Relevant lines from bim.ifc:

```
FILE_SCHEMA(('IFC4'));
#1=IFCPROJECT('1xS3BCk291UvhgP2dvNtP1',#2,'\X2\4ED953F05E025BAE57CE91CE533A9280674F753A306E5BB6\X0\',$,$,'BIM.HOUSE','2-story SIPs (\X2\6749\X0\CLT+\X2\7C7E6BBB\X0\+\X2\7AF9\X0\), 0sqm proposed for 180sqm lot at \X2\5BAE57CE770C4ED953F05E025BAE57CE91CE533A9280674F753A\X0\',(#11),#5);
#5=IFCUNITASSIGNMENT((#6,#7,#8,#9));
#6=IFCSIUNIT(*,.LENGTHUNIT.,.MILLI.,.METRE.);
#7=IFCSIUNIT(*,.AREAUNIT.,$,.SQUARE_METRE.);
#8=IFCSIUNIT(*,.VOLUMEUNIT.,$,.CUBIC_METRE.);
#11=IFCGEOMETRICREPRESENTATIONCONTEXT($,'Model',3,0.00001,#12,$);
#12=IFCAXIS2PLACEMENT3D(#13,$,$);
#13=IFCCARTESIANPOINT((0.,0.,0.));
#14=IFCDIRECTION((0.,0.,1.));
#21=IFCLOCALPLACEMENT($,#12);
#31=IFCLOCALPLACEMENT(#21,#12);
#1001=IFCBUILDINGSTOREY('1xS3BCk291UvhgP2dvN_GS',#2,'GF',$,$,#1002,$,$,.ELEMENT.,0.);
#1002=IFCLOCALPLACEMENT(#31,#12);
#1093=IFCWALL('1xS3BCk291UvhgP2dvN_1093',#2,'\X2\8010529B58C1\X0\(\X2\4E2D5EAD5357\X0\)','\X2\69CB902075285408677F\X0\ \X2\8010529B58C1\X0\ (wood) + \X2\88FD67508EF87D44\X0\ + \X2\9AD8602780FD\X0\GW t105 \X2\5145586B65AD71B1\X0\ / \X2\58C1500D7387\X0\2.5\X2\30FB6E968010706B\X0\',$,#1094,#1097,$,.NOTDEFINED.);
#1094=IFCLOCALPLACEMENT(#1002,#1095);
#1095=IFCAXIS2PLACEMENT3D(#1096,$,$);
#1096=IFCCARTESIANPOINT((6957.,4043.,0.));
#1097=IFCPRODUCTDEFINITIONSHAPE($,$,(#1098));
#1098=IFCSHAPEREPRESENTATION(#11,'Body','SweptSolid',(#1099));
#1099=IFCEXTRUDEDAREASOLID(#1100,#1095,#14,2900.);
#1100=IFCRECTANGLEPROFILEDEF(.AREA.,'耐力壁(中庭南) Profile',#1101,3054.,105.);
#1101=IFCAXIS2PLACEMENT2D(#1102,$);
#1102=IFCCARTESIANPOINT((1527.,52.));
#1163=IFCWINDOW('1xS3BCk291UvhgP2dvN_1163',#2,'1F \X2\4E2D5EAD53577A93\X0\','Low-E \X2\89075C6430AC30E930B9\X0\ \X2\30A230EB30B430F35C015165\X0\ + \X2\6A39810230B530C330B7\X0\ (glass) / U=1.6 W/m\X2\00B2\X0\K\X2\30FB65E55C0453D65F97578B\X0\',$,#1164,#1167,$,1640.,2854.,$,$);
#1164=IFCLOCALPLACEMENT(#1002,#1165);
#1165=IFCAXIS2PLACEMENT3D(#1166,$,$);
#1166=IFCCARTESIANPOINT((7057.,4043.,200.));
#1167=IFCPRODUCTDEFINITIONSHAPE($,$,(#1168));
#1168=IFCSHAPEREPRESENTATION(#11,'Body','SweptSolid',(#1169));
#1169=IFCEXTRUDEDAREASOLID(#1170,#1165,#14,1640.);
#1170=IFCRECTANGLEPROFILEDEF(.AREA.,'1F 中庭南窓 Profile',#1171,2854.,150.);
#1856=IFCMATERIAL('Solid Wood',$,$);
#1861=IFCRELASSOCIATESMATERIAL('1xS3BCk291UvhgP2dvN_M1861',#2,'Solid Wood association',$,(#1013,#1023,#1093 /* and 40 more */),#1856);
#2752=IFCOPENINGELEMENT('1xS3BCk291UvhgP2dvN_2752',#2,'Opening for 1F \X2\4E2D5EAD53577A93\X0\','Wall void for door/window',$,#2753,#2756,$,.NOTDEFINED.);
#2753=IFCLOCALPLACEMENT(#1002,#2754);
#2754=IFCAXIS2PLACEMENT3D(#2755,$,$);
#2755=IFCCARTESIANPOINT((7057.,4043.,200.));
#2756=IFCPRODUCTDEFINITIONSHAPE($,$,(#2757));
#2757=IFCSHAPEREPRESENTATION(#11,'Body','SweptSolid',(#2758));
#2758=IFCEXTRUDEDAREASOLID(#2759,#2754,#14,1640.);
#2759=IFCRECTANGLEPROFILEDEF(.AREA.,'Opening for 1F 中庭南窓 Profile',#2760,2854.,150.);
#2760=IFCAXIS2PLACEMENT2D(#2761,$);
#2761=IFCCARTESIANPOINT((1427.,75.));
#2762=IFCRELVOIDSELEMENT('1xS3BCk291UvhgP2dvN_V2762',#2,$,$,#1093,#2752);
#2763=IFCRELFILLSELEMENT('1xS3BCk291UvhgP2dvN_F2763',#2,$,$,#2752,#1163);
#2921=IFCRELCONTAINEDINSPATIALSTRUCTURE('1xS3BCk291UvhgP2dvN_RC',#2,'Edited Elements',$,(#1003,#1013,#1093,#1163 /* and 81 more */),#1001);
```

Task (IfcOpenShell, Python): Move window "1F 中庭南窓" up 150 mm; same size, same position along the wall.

```python
import numpy as np
import ifcopenshell
import ifcopenshell.api.geometry
import ifcopenshell.util.placement
import ifcopenshell.util.unit

model = ifcopenshell.open("bim.ifc")
unit_scale = ifcopenshell.util.unit.calculate_unit_scale(model)

window = model.by_guid("1xS3BCk291UvhgP2dvN_1163")
opening = window.FillsVoids[0].RelatingOpeningElement
dz = 0.15 / unit_scale

shift = np.array([0.0, 0.0, dz])
# The window is not placed relative to its opening, so move both.
for product in (opening, window):
    matrix = ifcopenshell.util.placement.get_local_placement(product.ObjectPlacement)
    matrix[:3, 3] += shift
    ifcopenshell.api.geometry.edit_object_placement(model, product=product, matrix=matrix, is_si=False)

print(f"moved by {dz * unit_scale:+.3f} m")

model.write("bim_v2.ifc")
```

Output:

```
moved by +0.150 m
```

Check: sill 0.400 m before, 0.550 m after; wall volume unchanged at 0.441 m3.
